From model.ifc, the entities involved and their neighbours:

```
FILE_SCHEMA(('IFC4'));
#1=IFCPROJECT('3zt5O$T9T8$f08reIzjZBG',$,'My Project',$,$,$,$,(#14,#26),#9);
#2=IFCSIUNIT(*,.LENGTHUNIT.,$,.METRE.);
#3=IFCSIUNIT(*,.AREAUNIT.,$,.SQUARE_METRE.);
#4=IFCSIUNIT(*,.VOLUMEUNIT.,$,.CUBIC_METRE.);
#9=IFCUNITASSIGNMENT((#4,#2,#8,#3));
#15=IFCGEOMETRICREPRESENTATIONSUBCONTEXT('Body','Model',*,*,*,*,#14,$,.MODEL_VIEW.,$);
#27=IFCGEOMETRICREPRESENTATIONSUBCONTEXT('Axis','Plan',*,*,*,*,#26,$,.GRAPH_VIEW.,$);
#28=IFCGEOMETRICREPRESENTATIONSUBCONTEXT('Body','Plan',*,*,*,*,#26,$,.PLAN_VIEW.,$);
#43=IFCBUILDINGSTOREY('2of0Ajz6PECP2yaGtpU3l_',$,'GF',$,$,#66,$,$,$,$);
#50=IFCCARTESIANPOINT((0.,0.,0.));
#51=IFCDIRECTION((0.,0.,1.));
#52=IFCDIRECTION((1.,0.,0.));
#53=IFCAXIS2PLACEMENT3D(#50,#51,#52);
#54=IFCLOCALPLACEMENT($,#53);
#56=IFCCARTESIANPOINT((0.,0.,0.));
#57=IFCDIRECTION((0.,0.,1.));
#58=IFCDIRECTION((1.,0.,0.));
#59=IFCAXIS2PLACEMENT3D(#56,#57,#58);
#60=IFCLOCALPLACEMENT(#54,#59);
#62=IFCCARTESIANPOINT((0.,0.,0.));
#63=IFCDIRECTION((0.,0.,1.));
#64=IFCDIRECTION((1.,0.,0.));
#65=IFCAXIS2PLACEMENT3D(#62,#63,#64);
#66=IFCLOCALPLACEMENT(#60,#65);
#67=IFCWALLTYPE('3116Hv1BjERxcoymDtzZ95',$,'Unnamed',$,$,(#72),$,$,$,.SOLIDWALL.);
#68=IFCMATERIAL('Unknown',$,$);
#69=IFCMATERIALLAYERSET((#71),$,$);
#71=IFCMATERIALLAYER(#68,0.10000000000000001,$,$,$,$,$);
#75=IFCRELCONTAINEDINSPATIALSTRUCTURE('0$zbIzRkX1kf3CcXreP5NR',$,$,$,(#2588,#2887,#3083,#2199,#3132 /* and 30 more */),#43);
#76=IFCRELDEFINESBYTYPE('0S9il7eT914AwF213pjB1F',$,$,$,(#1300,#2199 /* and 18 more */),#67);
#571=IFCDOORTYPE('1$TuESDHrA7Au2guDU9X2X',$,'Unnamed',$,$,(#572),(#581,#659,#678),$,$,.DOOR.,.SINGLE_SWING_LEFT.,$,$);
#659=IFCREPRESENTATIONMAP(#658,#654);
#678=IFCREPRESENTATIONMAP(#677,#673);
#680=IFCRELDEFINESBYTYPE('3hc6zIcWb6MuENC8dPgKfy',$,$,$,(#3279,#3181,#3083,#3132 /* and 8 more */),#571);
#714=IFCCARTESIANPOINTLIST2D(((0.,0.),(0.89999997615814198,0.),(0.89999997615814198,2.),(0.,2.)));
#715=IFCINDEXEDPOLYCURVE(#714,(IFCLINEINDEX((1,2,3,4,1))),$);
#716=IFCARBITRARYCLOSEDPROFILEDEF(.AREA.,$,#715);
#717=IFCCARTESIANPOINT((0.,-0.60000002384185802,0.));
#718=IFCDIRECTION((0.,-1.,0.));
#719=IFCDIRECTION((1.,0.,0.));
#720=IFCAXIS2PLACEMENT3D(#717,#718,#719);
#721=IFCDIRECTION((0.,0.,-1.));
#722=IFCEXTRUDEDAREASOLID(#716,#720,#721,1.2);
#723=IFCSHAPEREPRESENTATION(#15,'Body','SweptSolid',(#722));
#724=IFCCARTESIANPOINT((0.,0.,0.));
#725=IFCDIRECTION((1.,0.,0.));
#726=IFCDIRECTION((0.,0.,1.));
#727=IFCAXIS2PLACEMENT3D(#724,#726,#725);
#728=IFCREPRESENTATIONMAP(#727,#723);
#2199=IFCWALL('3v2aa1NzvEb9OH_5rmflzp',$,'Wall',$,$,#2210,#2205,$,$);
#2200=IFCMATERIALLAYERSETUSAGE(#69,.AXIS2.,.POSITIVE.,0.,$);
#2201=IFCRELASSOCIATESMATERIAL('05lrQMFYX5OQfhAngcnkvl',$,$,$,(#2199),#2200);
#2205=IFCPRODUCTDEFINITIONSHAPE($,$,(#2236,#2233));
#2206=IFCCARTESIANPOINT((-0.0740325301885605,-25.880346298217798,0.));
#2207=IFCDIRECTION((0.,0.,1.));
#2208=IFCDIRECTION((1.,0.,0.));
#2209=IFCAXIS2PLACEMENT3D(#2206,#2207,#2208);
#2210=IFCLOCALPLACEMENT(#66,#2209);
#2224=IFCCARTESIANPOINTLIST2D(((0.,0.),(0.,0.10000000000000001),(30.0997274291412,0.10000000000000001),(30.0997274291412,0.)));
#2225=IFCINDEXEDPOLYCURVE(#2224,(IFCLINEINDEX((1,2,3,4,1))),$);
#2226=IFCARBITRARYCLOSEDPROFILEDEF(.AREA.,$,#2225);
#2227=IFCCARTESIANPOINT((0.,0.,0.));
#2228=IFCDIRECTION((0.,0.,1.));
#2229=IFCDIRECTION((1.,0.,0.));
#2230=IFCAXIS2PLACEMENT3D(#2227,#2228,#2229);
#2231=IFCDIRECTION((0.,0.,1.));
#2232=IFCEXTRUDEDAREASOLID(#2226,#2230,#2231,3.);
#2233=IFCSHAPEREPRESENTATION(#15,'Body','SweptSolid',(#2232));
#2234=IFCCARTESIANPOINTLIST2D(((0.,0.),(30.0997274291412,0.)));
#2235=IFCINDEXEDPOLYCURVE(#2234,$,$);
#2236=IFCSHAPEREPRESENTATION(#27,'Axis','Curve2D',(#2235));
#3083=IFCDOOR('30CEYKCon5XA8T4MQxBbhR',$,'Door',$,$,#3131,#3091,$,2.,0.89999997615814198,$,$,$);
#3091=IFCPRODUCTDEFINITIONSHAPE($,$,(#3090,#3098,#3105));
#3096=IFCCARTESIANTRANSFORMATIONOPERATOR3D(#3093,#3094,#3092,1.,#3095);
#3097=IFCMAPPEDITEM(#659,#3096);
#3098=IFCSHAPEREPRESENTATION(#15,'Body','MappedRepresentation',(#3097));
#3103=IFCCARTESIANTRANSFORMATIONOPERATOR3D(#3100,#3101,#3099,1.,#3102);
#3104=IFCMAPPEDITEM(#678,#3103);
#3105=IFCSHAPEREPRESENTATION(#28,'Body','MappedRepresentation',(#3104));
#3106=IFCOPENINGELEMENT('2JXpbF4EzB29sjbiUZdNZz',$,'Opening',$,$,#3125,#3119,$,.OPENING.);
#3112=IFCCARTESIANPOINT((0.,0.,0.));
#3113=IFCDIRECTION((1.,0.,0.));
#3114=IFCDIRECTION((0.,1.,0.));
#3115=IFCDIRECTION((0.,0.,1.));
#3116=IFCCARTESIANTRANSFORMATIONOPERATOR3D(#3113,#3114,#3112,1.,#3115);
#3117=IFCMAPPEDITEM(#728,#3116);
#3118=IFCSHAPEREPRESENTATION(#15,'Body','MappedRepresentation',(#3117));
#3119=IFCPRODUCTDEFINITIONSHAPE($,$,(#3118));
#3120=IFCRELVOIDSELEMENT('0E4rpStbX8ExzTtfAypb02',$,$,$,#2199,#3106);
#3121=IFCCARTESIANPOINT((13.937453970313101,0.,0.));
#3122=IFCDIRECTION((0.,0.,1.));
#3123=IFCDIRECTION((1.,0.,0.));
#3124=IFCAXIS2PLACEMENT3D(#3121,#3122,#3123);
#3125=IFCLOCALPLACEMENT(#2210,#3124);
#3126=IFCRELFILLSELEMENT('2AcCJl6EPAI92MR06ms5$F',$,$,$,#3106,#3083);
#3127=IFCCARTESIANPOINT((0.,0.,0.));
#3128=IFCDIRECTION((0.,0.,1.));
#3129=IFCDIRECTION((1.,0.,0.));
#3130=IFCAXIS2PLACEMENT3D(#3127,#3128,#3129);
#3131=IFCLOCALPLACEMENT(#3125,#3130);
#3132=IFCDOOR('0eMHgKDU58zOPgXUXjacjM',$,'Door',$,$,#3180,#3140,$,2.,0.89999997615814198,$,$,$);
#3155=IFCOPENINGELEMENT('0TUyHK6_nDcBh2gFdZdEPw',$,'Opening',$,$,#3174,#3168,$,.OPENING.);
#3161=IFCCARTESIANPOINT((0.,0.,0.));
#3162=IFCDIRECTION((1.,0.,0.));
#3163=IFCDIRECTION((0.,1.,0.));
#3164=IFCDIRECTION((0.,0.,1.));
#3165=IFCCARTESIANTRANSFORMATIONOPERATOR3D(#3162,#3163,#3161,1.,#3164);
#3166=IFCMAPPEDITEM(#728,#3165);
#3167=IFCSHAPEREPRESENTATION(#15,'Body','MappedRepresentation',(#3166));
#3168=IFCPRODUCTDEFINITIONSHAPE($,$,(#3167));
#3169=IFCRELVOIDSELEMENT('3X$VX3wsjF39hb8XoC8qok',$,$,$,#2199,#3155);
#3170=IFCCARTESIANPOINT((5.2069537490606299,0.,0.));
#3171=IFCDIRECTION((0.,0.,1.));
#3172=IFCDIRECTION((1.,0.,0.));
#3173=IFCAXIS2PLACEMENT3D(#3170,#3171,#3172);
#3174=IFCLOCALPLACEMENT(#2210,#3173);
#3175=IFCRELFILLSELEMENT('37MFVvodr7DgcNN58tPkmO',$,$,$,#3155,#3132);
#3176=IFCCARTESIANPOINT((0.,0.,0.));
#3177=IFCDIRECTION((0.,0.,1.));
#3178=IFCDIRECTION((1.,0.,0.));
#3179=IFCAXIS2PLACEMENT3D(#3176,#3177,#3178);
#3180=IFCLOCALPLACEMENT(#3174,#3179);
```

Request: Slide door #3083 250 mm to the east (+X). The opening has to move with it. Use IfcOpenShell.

```python
import ifcopenshell
import ifcopenshell.api.geometry
import ifcopenshell.util.placement

model = ifcopenshell.open("model.ifc")

door = model.by_guid("30CEYKCon5XA8T4MQxBbhR")
opening = door.FillsVoids[0].RelatingOpeningElement
wall = opening.VoidsElements[0].RelatingBuildingElement

wall_matrix = ifcopenshell.util.placement.get_local_placement(wall.ObjectPlacement)
shift = wall_matrix[:3, 0] * 0.25
before = ifcopenshell.util.placement.get_local_placement(door.ObjectPlacement)[:3, 3].copy()

# The door is placed relative to its opening, so it follows when the opening moves.
matrix = ifcopenshell.util.placement.get_local_placement(opening.ObjectPlacement)
matrix[:3, 3] += shift
ifcopenshell.api.geometry.edit_object_placement(
    model, product=opening, matrix=matrix, is_si=False, should_transform_children=True
)

after = ifcopenshell.util.placement.get_local_placement(door.ObjectPlacement)[:3, 3]
print("door moved by", (after - before).round(3) + 0.0)

model.write("model_rev.ifc")
```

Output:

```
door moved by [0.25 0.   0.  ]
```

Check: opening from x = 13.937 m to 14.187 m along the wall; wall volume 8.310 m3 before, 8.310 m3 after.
